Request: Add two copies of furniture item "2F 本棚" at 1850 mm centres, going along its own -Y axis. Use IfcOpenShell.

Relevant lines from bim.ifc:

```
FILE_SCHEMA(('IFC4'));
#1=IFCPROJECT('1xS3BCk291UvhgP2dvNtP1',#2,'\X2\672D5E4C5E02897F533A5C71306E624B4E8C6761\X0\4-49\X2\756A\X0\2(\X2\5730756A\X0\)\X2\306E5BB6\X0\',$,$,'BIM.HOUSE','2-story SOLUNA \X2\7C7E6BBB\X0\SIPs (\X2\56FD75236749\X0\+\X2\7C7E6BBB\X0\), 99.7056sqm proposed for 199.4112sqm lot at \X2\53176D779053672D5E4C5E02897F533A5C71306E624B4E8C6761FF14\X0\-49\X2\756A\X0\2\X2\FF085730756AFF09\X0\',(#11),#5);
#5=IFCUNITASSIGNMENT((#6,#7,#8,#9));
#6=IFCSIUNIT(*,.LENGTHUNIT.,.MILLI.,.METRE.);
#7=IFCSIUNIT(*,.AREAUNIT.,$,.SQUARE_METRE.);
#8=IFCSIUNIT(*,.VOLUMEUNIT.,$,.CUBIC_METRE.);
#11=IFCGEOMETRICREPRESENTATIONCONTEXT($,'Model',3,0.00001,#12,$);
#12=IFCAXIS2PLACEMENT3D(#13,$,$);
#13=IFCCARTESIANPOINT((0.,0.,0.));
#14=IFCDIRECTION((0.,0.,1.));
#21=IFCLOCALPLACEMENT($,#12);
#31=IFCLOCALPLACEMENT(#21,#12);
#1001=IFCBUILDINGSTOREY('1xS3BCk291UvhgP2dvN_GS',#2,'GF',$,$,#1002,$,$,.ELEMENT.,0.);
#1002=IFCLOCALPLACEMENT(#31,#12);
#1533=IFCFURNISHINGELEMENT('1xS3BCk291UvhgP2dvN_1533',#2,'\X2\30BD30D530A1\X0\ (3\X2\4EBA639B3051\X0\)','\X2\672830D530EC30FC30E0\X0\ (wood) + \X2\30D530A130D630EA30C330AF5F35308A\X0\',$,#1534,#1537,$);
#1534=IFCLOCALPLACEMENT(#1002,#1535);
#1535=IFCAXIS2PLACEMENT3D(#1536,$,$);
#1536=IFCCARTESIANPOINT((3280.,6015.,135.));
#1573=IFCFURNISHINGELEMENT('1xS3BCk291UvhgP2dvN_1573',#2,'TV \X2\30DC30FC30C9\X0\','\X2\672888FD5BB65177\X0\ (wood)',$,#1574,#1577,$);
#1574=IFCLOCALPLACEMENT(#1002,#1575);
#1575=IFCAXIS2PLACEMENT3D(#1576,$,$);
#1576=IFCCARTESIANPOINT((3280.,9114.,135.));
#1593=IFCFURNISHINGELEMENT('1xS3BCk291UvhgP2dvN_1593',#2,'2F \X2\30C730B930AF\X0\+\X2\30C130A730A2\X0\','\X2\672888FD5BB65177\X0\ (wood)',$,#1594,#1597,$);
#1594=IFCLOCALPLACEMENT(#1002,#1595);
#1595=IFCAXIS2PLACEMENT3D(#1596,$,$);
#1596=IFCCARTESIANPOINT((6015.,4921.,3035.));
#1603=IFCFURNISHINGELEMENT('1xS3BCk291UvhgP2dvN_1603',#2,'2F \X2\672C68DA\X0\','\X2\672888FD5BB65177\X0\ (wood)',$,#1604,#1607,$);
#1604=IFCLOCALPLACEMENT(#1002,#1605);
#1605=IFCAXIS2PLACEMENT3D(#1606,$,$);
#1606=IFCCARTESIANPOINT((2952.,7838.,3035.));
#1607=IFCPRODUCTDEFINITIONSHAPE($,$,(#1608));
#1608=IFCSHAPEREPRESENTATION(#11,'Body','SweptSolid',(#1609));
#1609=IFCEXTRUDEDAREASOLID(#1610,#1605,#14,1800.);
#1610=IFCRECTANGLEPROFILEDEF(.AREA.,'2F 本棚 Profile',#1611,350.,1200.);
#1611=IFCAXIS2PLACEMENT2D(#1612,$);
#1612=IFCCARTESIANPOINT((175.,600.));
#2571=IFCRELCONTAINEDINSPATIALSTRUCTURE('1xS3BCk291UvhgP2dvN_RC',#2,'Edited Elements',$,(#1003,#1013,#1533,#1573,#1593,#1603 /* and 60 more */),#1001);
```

```python
import ifcopenshell
import ifcopenshell.api.geometry
import ifcopenshell.api.root
import ifcopenshell.util.element
import ifcopenshell.util.placement
import ifcopenshell.util.unit

model = ifcopenshell.open("bim.ifc")
unit_scale = ifcopenshell.util.unit.calculate_unit_scale(model)


def reuse_history(source, copy):
    """copy_class also copies each property set's owner history, people and application; keep the originals."""
    for rel in copy.IsDefinedBy:
        if rel.is_a("IfcRelDefinesByProperties") and (history := rel.RelatingPropertyDefinition.OwnerHistory):
            rel.RelatingPropertyDefinition.OwnerHistory = source.OwnerHistory
            ifcopenshell.util.element.remove_deep2(model, history)


source = model.by_guid("1xS3BCk291UvhgP2dvN_1603")
base = ifcopenshell.util.placement.get_local_placement(source.ObjectPlacement)
step = -base[:3, 1] * 1.85 / unit_scale

for i in range(1, 3):
    copy = ifcopenshell.api.root.copy_class(model, product=source)
    copy.Representation = ifcopenshell.util.element.copy_deep(
        model, source.Representation, exclude=["IfcGeometricRepresentationContext", "IfcRepresentationMap"]
    )
    reuse_history(source, copy)
    matrix = base.copy()
    matrix[:3, 3] += i * step
    print("added at", matrix[:3, 3].round(3) + 0.0)
    ifcopenshell.api.geometry.edit_object_placement(model, product=copy, matrix=matrix, is_si=False)

model.write("bim_updated.ifc")
```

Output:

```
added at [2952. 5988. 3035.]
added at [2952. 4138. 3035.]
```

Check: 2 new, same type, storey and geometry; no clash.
